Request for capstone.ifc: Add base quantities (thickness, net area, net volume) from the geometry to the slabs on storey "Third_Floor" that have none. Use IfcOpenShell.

First a look at what the model holds.

```python
import ifcopenshell
import ifcopenshell.util.element
import ifcopenshell.util.unit

model = ifcopenshell.open("capstone.ifc")
print(model.schema)
for unit_type in ("LENGTHUNIT", "AREAUNIT", "VOLUMEUNIT"):
    print(unit_type, ifcopenshell.util.unit.calculate_unit_scale(model, unit_type))
storey = next(s for s in model.by_type("IfcBuildingStorey") if s.Name == "Third_Floor")
slabs = [e for e in ifcopenshell.util.element.get_decomposition(storey) if e.is_a("IfcSlab")]
for e in sorted(slabs, key=lambda e: e.id()):
    print(e.id(), e.is_a(), e.Name, list(ifcopenshell.util.element.get_psets(e, qtos_only=True)), sep=" | ")
```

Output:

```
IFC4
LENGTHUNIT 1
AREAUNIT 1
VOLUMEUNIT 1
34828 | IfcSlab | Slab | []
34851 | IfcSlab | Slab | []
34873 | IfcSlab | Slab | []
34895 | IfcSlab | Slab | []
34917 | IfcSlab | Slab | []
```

```python
import ifcopenshell
import ifcopenshell.api.pset
import ifcopenshell.geom
import ifcopenshell.util.element
import ifcopenshell.util.shape
import ifcopenshell.util.unit

model = ifcopenshell.open("capstone.ifc")
unit_scale = ifcopenshell.util.unit.calculate_unit_scale(model)
area_scale = ifcopenshell.util.unit.calculate_unit_scale(model, "AREAUNIT")
volume_scale = ifcopenshell.util.unit.calculate_unit_scale(model, "VOLUMEUNIT")
settings = ifcopenshell.geom.settings()

storey = next(s for s in model.by_type("IfcBuildingStorey") if s.Name == "Third_Floor")
slabs = [e for e in ifcopenshell.util.element.get_decomposition(storey) if e.is_a("IfcSlab")]

for e in sorted(slabs, key=lambda e: e.id()):
    if ifcopenshell.util.element.get_psets(e, qtos_only=True, should_inherit=False):
        continue
    # Geometry comes back in metres, in the element's own axes.
    shape = ifcopenshell.geom.create_shape(settings, e)
    values = {
        "Width": ifcopenshell.util.shape.get_z(shape.geometry) / unit_scale,
        "NetArea": ifcopenshell.util.shape.get_footprint_area(shape.geometry) / area_scale,
        "NetVolume": ifcopenshell.util.shape.get_volume(shape.geometry) / volume_scale,
    }
    qto = ifcopenshell.api.pset.add_qto(model, product=e, name="Qto_SlabBaseQuantities")
    ifcopenshell.api.pset.edit_qto(model, qto=qto, properties=values)
    print(e.id(), {k: round(v, 3) for k, v in values.items()})

model.write("capstone-out.ifc")
```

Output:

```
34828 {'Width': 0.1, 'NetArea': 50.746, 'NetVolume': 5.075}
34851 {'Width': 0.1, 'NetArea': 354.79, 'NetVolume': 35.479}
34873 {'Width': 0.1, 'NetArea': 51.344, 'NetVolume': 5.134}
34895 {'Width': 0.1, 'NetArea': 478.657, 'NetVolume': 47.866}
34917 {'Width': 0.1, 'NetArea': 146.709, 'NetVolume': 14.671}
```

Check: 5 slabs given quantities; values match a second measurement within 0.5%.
